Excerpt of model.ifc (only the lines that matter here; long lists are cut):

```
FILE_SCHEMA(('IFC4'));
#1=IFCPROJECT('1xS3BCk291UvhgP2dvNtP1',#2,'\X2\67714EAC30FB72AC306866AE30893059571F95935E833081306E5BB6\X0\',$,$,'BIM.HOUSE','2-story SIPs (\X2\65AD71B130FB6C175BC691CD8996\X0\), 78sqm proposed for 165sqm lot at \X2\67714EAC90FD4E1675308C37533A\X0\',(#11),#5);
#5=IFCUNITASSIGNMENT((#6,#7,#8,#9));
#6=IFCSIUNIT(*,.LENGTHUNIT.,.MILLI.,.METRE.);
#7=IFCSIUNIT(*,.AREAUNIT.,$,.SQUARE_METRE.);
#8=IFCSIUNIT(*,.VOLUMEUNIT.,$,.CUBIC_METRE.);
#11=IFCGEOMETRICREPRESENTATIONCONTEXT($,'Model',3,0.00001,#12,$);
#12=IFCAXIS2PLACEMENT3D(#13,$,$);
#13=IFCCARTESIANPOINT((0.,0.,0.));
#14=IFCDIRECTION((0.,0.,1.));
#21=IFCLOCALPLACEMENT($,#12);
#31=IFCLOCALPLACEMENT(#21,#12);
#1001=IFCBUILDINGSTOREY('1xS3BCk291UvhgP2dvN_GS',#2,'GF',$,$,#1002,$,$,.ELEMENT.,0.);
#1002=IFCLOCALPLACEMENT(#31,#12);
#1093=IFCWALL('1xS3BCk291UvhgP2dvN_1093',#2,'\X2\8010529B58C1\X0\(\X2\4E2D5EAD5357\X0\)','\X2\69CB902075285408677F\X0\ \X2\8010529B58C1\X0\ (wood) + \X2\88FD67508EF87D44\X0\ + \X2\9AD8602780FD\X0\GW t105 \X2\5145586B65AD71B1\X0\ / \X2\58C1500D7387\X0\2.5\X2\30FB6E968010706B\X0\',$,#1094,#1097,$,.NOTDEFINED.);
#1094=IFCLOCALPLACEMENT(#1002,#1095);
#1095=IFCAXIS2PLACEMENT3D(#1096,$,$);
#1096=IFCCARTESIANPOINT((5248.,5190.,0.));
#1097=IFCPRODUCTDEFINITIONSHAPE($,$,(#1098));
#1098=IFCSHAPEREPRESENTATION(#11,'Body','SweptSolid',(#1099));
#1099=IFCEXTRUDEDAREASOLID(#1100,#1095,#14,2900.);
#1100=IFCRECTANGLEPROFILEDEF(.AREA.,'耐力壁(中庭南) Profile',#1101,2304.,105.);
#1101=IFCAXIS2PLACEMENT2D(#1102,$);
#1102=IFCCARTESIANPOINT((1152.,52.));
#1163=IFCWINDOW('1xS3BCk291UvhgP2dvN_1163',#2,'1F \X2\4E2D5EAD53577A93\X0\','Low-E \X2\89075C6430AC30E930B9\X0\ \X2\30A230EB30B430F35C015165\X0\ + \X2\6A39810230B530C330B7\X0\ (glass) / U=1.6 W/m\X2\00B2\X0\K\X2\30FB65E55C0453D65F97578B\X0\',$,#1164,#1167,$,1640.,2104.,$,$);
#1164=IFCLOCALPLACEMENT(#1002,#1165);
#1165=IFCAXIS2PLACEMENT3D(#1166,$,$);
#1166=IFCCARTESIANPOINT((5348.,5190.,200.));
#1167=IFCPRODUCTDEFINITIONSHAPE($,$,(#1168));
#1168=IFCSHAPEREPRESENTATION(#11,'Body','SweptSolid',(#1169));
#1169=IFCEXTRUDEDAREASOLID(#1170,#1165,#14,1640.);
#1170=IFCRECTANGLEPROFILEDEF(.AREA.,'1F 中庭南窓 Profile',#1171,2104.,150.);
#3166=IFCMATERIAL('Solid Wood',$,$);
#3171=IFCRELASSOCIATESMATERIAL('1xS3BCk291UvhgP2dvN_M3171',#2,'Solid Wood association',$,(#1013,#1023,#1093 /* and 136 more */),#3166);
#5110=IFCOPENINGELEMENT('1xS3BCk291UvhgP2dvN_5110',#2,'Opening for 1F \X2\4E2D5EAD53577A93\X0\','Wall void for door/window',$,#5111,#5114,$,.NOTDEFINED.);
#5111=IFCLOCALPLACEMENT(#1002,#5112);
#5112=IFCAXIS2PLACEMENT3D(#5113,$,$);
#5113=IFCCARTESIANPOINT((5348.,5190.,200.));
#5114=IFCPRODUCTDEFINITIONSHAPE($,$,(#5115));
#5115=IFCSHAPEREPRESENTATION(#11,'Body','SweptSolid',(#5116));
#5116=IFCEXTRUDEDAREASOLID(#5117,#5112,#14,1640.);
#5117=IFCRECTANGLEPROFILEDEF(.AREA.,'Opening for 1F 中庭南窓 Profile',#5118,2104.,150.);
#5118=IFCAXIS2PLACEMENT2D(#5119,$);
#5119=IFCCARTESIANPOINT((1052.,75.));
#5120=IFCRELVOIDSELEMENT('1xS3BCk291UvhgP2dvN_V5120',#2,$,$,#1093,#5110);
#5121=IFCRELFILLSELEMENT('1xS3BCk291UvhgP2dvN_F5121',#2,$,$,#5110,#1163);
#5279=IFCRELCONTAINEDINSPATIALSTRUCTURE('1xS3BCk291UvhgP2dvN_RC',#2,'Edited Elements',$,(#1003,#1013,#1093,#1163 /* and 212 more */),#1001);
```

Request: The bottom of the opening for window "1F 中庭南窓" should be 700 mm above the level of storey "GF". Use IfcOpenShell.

```python
import numpy as np
import ifcopenshell
import ifcopenshell.api.geometry
import ifcopenshell.geom
import ifcopenshell.util.element
import ifcopenshell.util.placement
import ifcopenshell.util.shape
import ifcopenshell.util.unit

model = ifcopenshell.open("model.ifc")
unit_scale = ifcopenshell.util.unit.calculate_unit_scale(model)

window = model.by_id(1163)
opening = window.FillsVoids[0].RelatingOpeningElement
storey = ifcopenshell.util.element.get_container(window, ifc_class="IfcBuildingStorey")
level = ifcopenshell.util.placement.get_local_placement(storey.ObjectPlacement)[2, 3]

# The opening's origin need not be at the sill, so measure its lowest point.
shape = ifcopenshell.geom.create_shape(ifcopenshell.geom.settings(), opening)
bottom = ifcopenshell.util.shape.get_shape_bottom_elevation(shape, shape.geometry) / unit_scale
dz = level + 0.7 / unit_scale - bottom

shift = np.array([0.0, 0.0, dz])
# The window is not placed relative to its opening, so move both.
for product in (opening, window):
    matrix = ifcopenshell.util.placement.get_local_placement(product.ObjectPlacement)
    matrix[:3, 3] += shift
    ifcopenshell.api.geometry.edit_object_placement(model, product=product, matrix=matrix, is_si=False)

print(f"moved by {dz * unit_scale:+.3f} m")

model.write("model_updated.ifc")
```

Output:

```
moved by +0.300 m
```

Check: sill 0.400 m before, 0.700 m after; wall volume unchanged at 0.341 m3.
